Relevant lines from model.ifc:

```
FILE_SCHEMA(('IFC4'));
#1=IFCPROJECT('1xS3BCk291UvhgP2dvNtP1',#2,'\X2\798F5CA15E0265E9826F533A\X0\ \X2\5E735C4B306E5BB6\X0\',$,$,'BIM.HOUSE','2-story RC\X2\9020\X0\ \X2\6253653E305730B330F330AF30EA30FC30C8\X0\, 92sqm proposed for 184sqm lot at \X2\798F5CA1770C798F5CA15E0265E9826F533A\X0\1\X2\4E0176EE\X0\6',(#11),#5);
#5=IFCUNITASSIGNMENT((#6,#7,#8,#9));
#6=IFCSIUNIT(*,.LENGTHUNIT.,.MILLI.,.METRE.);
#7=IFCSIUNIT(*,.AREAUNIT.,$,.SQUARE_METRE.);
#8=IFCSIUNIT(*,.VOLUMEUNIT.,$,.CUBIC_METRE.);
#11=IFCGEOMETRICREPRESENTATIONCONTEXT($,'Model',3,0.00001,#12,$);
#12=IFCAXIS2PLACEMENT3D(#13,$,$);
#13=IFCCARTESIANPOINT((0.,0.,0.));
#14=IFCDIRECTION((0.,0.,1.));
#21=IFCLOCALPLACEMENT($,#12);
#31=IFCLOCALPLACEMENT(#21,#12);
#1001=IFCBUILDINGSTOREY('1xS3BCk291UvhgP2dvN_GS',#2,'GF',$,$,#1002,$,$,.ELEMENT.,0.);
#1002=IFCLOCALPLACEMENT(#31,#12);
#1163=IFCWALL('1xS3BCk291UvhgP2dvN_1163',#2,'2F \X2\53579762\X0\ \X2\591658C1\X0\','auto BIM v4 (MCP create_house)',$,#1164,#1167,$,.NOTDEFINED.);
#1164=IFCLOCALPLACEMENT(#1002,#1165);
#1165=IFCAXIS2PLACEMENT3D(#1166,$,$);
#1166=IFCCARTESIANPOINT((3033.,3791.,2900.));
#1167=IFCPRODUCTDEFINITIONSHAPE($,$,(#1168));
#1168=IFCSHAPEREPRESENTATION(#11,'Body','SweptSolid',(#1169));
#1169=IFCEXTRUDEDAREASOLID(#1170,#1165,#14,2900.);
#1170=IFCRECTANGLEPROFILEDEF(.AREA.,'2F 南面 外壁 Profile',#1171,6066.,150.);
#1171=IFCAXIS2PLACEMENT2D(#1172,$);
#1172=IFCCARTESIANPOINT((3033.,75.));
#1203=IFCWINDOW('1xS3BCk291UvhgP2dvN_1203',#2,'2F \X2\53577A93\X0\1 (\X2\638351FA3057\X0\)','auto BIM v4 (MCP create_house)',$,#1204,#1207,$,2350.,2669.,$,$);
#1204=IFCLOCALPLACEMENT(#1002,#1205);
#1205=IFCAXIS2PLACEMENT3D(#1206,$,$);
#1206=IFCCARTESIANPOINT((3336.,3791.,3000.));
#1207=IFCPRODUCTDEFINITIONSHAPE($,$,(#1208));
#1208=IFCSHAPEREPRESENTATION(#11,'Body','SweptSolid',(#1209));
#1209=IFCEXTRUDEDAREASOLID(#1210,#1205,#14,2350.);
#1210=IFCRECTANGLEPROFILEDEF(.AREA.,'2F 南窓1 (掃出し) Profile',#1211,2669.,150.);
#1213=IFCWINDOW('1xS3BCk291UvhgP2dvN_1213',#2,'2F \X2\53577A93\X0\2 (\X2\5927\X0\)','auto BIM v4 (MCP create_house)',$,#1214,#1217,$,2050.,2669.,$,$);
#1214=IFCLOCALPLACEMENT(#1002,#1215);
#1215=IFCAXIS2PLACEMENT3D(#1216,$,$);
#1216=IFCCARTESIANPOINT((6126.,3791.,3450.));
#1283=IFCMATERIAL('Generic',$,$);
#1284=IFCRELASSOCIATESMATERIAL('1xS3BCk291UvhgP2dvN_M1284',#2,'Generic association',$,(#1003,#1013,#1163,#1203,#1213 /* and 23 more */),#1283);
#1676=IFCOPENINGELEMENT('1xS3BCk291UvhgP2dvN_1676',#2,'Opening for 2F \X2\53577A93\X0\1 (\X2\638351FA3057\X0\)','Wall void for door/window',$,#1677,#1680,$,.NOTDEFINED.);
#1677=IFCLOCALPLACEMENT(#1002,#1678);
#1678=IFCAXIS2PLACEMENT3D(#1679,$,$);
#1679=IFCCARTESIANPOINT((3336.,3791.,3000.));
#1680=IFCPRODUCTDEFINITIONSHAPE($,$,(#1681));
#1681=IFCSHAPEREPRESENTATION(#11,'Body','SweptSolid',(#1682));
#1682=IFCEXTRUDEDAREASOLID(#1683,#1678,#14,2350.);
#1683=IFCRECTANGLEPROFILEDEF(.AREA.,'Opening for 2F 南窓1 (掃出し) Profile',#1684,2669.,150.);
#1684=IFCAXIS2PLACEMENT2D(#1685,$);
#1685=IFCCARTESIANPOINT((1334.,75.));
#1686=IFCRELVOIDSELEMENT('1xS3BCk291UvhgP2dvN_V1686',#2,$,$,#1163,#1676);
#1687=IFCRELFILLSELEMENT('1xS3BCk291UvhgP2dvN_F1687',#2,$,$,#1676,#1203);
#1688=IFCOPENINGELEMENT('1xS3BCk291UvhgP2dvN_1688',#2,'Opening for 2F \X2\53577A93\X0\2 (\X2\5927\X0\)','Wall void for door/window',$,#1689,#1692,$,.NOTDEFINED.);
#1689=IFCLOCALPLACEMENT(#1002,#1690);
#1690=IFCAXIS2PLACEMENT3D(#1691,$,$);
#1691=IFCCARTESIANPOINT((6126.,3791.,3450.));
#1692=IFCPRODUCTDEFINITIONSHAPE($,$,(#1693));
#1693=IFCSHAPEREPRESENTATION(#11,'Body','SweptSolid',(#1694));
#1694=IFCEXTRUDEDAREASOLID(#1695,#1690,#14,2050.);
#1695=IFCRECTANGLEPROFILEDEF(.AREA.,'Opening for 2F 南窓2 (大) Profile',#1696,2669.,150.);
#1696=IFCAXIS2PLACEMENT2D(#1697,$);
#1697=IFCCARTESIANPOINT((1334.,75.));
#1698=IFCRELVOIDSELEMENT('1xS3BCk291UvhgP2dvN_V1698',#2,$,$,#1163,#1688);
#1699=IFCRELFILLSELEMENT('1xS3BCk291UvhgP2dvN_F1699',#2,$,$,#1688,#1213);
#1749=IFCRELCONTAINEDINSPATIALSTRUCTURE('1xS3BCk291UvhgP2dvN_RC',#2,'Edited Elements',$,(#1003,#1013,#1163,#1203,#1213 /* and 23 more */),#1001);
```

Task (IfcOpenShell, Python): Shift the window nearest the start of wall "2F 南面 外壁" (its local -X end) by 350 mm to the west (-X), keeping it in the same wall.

```python
import ifcopenshell
import ifcopenshell.api.geometry
import ifcopenshell.util.placement

model = ifcopenshell.open("model.ifc")

window = model.by_guid("1xS3BCk291UvhgP2dvN_1203")
opening = window.FillsVoids[0].RelatingOpeningElement
wall = opening.VoidsElements[0].RelatingBuildingElement

wall_matrix = ifcopenshell.util.placement.get_local_placement(wall.ObjectPlacement)
shift = wall_matrix[:3, 0] * -350.0
before = ifcopenshell.util.placement.get_local_placement(window.ObjectPlacement)[:3, 3].copy()

# The window is not placed relative to its opening, so move both.
for product in (opening, window):
    matrix = ifcopenshell.util.placement.get_local_placement(product.ObjectPlacement)
    matrix[:3, 3] += shift
    ifcopenshell.api.geometry.edit_object_placement(model, product=product, matrix=matrix, is_si=False)

after = ifcopenshell.util.placement.get_local_placement(window.ObjectPlacement)[:3, 3]
print("window moved by", (after - before).round(3) + 0.0)

model.write("model-out.ifc")
```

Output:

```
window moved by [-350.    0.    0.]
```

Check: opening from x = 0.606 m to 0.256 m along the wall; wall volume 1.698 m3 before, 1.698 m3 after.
